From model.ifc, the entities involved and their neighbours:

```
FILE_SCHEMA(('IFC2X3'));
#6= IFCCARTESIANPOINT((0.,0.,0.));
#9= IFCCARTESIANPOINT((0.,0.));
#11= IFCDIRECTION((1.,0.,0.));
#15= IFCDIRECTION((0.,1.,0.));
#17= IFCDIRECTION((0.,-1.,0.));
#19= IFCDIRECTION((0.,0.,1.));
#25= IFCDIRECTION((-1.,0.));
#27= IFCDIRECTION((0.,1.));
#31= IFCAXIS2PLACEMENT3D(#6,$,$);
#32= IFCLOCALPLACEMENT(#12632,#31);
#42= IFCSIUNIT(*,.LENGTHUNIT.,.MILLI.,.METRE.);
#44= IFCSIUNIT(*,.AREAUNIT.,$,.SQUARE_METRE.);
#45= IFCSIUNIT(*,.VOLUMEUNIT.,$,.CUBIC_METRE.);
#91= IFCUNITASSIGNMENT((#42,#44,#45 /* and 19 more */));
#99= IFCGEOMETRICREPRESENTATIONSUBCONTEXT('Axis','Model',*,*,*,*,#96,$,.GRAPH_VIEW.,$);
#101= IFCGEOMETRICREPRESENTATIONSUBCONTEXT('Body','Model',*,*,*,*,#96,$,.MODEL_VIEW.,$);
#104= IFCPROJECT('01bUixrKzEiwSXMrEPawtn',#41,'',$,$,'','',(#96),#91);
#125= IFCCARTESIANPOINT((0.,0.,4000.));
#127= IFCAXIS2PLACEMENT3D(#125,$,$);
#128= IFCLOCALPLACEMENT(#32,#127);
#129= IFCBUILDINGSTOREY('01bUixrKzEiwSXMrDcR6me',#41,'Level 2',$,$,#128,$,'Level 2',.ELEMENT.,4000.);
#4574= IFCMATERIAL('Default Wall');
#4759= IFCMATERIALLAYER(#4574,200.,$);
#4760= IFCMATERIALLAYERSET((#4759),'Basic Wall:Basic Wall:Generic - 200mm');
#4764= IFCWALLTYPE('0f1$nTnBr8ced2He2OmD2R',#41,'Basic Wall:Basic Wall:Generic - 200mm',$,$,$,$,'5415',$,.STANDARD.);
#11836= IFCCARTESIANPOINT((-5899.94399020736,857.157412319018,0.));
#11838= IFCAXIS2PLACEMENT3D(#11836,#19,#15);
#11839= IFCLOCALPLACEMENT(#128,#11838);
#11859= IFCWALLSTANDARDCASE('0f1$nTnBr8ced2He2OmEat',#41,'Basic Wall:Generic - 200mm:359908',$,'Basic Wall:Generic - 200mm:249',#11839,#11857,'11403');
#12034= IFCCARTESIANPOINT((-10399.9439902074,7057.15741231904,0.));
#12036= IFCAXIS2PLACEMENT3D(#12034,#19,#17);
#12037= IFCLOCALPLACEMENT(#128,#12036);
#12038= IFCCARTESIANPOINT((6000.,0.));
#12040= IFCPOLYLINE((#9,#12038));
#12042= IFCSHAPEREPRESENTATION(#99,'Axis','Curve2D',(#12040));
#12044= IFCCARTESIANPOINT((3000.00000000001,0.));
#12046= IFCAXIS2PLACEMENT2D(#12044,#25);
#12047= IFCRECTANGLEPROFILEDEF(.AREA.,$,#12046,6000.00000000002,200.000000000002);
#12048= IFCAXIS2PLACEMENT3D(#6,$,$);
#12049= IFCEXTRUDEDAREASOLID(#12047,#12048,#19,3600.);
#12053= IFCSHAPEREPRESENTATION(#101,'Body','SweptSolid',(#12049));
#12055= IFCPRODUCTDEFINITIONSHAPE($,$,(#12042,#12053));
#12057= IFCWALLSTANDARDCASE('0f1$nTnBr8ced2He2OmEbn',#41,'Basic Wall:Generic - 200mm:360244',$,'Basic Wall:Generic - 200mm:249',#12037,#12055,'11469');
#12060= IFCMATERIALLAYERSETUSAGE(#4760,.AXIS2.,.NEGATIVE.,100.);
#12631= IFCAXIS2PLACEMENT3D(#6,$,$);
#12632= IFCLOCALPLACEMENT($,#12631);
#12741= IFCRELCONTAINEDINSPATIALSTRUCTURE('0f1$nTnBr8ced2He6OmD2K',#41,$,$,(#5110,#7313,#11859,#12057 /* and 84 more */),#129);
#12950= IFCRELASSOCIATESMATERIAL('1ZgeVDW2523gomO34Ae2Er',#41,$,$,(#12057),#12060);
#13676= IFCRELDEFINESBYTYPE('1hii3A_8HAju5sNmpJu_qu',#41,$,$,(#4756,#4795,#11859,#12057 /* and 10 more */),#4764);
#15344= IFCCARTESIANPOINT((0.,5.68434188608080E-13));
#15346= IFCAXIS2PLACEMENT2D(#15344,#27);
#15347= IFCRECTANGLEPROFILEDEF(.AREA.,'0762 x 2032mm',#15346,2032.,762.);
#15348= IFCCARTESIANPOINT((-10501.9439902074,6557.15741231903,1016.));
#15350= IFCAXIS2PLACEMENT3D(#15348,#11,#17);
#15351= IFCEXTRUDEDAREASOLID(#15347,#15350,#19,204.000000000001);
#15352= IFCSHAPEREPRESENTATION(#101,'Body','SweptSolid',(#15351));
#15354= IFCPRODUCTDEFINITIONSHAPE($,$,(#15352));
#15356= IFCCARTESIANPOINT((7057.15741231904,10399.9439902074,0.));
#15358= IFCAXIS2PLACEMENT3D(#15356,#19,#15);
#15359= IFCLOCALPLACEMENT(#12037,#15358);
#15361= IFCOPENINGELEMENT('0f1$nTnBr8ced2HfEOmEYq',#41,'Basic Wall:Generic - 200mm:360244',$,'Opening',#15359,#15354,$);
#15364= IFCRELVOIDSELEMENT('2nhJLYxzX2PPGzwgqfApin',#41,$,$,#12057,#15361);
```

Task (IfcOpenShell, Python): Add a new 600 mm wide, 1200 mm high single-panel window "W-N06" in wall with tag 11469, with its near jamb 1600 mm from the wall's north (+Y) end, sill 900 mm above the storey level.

```python
import numpy as np
import ifcopenshell
import ifcopenshell.api.feature
import ifcopenshell.api.geometry
import ifcopenshell.api.root
import ifcopenshell.api.spatial
import ifcopenshell.api.type
import ifcopenshell.geom
import ifcopenshell.util.element
import ifcopenshell.util.placement
import ifcopenshell.util.representation
import ifcopenshell.util.shape
import ifcopenshell.util.unit

model = ifcopenshell.open("model.ifc")
unit_scale = ifcopenshell.util.unit.calculate_unit_scale(model)
settings = ifcopenshell.geom.settings()


def volume(element):
    """Net volume in cubic metres, openings subtracted."""
    shape = ifcopenshell.geom.create_shape(settings, element)
    return ifcopenshell.util.shape.get_volume(shape.geometry)


wall = model.by_guid("0f1$nTnBr8ced2He2OmEbn")
storey = ifcopenshell.util.element.get_container(wall, ifc_class="IfcBuildingStorey")
context = ifcopenshell.util.representation.get_context(model, "Model", "Body", "MODEL_VIEW")
before = volume(wall)

width, height, from_end, sill = 0.6, 1.2, 1.6, 0.9  # metres

# The wall runs along its own X axis, and the end named is its -X end.
wall_shape = ifcopenshell.geom.create_shape(settings, wall)
x, y, z = ifcopenshell.util.shape.get_vertices(wall_shape.geometry).T
start = x.min() + from_end
face, thickness = float(y.min()), float(y.max() - y.min())
wall_matrix = ifcopenshell.util.placement.get_local_placement(wall.ObjectPlacement)
level = ifcopenshell.util.placement.get_local_placement(storey.ObjectPlacement)[2, 3]


def in_wall(x, y):
    """Placement at x, y metres in the wall's axes, at sill height."""
    matrix = wall_matrix.copy()
    matrix[:, 3] = wall_matrix @ np.array([x / unit_scale, y / unit_scale, 0.0, 1.0])
    matrix[2, 3] = level + sill / unit_scale
    return matrix


# Opening: a box that overshoots both wall faces by 50 mm.
opening = ifcopenshell.api.root.create_entity(model, ifc_class="IfcOpeningElement")
box = ifcopenshell.api.geometry.add_wall_representation(
    model, context=context, length=width, height=height, thickness=thickness + 0.1
)
ifcopenshell.api.geometry.assign_representation(model, product=opening, representation=box)
ifcopenshell.api.geometry.edit_object_placement(model, product=opening, matrix=in_wall(start, face - 0.05), is_si=False)
ifcopenshell.api.feature.add_feature(model, feature=opening, element=wall)

window = ifcopenshell.api.root.create_entity(model, ifc_class="IfcWindow", name="W-N06")
window.OverallWidth, window.OverallHeight = width / unit_scale, height / unit_scale
body = ifcopenshell.api.geometry.add_window_representation(
    model,
    context=context,
    overall_width=window.OverallWidth,
    overall_height=window.OverallHeight,
    partition_type="SINGLE_PANEL",
)
ifcopenshell.api.geometry.assign_representation(model, product=window, representation=body)
ifcopenshell.api.spatial.assign_container(model, products=[window], relating_structure=storey)
fills = ifcopenshell.api.feature.add_filling(model, opening=opening, element=window)
fills.OwnerHistory = window.OwnerHistory  # required in IFC2X3

# IFC2X3 keeps the operation on the window style.
style = ifcopenshell.api.root.create_entity(model, ifc_class="IfcWindowStyle", name="W-N06")
style.OperationType, style.ConstructionType = "SINGLE_PANEL", "NOTDEFINED"
style.ParameterTakesPrecedence = style.Sizeable = False
ifcopenshell.api.type.assign_type(model, related_objects=[window], relating_type=style)

# Centre the window in the wall's thickness.
ifcopenshell.api.geometry.edit_object_placement(model, product=window, matrix=in_wall(start, face), is_si=False)
window_shape = ifcopenshell.geom.create_shape(settings, window)
depth = ifcopenshell.util.shape.get_vertices(window_shape.geometry)[:, 1]
offset = face + thickness / 2 - (depth.min() + depth.max()) / 2
ifcopenshell.api.geometry.edit_object_placement(model, product=window, matrix=in_wall(start, offset), is_si=False)

after = volume(wall)

print(f"wall volume {before:.3f} -> {after:.3f} m3")

model.write("model_edited.ifc")
```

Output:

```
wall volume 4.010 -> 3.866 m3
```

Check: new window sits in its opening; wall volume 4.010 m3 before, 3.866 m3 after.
